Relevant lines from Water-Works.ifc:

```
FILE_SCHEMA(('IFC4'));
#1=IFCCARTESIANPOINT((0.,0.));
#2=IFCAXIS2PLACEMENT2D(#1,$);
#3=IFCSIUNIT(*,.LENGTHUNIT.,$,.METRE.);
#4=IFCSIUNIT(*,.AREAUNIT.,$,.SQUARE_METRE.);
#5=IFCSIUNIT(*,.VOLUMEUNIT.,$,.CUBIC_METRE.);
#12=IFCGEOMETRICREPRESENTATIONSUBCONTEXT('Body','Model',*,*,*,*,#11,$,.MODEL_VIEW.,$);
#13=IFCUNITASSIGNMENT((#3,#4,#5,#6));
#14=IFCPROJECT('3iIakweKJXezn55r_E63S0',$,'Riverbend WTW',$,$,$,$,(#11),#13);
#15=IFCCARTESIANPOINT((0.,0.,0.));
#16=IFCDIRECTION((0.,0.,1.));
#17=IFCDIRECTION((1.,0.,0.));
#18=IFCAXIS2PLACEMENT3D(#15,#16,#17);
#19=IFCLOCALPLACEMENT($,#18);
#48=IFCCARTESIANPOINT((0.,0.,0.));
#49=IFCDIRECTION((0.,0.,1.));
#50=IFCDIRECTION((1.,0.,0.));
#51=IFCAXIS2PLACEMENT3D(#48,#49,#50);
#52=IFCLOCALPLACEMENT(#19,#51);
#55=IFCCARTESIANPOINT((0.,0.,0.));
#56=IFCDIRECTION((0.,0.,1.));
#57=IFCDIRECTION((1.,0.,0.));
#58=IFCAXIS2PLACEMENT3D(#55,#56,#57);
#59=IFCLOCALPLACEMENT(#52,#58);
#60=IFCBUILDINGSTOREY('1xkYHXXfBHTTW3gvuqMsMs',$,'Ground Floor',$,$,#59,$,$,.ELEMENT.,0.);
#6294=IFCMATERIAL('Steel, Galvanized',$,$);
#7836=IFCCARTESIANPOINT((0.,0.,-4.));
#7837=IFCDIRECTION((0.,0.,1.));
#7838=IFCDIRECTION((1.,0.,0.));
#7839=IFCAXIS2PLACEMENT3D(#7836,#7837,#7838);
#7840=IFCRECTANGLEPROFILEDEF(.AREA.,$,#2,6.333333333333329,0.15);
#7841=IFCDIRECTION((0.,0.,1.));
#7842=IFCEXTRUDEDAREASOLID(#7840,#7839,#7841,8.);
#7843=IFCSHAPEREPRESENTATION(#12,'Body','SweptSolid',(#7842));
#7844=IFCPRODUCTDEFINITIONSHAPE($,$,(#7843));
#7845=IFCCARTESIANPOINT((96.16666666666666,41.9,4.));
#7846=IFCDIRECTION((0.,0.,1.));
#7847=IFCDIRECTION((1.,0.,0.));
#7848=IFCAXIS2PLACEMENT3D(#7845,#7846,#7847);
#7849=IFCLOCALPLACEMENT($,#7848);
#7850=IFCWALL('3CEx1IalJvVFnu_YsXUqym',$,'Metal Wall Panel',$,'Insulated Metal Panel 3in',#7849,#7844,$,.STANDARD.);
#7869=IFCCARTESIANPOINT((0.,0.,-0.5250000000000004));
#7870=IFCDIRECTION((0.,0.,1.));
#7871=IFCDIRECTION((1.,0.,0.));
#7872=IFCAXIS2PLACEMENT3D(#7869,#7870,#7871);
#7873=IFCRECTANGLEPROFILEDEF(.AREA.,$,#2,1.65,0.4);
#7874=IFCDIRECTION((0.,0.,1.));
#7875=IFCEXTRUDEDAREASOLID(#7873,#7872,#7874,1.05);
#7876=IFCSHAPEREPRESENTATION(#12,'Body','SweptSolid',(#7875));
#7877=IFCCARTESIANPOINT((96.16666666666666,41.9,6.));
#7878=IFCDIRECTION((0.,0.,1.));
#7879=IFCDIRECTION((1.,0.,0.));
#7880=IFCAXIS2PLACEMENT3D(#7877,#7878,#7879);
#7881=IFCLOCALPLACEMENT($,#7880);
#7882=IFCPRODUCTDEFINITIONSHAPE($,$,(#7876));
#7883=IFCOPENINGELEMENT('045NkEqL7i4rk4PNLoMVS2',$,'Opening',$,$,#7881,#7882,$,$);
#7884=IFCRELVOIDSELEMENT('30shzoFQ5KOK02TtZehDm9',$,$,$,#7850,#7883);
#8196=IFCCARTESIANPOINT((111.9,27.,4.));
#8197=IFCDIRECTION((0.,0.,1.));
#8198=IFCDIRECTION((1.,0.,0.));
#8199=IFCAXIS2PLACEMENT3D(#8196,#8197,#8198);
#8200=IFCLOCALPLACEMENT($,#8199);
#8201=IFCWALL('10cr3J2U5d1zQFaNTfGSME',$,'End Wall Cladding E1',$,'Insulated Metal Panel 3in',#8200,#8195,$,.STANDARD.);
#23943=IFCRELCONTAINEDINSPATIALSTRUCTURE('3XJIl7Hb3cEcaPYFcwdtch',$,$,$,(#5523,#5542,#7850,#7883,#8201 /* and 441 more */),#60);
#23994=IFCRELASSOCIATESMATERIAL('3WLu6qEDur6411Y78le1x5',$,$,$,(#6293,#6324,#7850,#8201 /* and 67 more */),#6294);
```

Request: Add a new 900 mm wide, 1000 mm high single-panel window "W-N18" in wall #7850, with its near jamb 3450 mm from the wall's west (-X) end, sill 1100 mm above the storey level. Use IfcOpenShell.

```python
import numpy as np
import ifcopenshell
import ifcopenshell.api.feature
import ifcopenshell.api.geometry
import ifcopenshell.api.root
import ifcopenshell.api.spatial
import ifcopenshell.geom
import ifcopenshell.util.element
import ifcopenshell.util.placement
import ifcopenshell.util.representation
import ifcopenshell.util.shape
import ifcopenshell.util.unit

model = ifcopenshell.open("Water-Works.ifc")
unit_scale = ifcopenshell.util.unit.calculate_unit_scale(model)
settings = ifcopenshell.geom.settings()


def volume(element):
    """Net volume in cubic metres, openings subtracted."""
    shape = ifcopenshell.geom.create_shape(settings, element)
    return ifcopenshell.util.shape.get_volume(shape.geometry)


wall = model.by_id(7850)
storey = ifcopenshell.util.element.get_container(wall, ifc_class="IfcBuildingStorey")
context = ifcopenshell.util.representation.get_context(model, "Model", "Body", "MODEL_VIEW")
before = volume(wall)

width, height, from_end, sill = 0.9, 1, 3.45, 1.1  # metres

# The wall runs along its own X axis, and the end named is its -X end.
wall_shape = ifcopenshell.geom.create_shape(settings, wall)
x, y, z = ifcopenshell.util.shape.get_vertices(wall_shape.geometry).T
start = x.min() + from_end
face, thickness = float(y.min()), float(y.max() - y.min())
wall_matrix = ifcopenshell.util.placement.get_local_placement(wall.ObjectPlacement)
level = ifcopenshell.util.placement.get_local_placement(storey.ObjectPlacement)[2, 3]


def in_wall(x, y):
    """Placement at x, y metres in the wall's axes, at sill height."""
    matrix = wall_matrix.copy()
    matrix[:, 3] = wall_matrix @ np.array([x / unit_scale, y / unit_scale, 0.0, 1.0])
    matrix[2, 3] = level + sill / unit_scale
    return matrix


# Opening: a box that overshoots both wall faces by 50 mm.
opening = ifcopenshell.api.root.create_entity(model, ifc_class="IfcOpeningElement", predefined_type="OPENING")
box = ifcopenshell.api.geometry.add_wall_representation(
    model, context=context, length=width, height=height, thickness=thickness + 0.1
)
ifcopenshell.api.geometry.assign_representation(model, product=opening, representation=box)
ifcopenshell.api.geometry.edit_object_placement(model, product=opening, matrix=in_wall(start, face - 0.05), is_si=False)
ifcopenshell.api.feature.add_feature(model, feature=opening, element=wall)

window = ifcopenshell.api.root.create_entity(model, ifc_class="IfcWindow", name="W-N18", predefined_type="WINDOW")
window.OverallWidth, window.OverallHeight = width / unit_scale, height / unit_scale
window.PartitioningType = "SINGLE_PANEL"
body = ifcopenshell.api.geometry.add_window_representation(
    model,
    context=context,
    overall_width=window.OverallWidth,
    overall_height=window.OverallHeight,
    partition_type="SINGLE_PANEL",
)
ifcopenshell.api.geometry.assign_representation(model, product=window, representation=body)
ifcopenshell.api.spatial.assign_container(model, products=[window], relating_structure=storey)
ifcopenshell.api.feature.add_filling(model, opening=opening, element=window)

# Centre the window in the wall's thickness.
ifcopenshell.api.geometry.edit_object_placement(model, product=window, matrix=in_wall(start, face), is_si=False)
window_shape = ifcopenshell.geom.create_shape(settings, window)
depth = ifcopenshell.util.shape.get_vertices(window_shape.geometry)[:, 1]
offset = face + thickness / 2 - (depth.min() + depth.max()) / 2
ifcopenshell.api.geometry.edit_object_placement(model, product=window, matrix=in_wall(start, offset), is_si=False)

after = volume(wall)

print(f"wall volume {before:.3f} -> {after:.3f} m3")

model.write("Water-Works_updated.ifc")
```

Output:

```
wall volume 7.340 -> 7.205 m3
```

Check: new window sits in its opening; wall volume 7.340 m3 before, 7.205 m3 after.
